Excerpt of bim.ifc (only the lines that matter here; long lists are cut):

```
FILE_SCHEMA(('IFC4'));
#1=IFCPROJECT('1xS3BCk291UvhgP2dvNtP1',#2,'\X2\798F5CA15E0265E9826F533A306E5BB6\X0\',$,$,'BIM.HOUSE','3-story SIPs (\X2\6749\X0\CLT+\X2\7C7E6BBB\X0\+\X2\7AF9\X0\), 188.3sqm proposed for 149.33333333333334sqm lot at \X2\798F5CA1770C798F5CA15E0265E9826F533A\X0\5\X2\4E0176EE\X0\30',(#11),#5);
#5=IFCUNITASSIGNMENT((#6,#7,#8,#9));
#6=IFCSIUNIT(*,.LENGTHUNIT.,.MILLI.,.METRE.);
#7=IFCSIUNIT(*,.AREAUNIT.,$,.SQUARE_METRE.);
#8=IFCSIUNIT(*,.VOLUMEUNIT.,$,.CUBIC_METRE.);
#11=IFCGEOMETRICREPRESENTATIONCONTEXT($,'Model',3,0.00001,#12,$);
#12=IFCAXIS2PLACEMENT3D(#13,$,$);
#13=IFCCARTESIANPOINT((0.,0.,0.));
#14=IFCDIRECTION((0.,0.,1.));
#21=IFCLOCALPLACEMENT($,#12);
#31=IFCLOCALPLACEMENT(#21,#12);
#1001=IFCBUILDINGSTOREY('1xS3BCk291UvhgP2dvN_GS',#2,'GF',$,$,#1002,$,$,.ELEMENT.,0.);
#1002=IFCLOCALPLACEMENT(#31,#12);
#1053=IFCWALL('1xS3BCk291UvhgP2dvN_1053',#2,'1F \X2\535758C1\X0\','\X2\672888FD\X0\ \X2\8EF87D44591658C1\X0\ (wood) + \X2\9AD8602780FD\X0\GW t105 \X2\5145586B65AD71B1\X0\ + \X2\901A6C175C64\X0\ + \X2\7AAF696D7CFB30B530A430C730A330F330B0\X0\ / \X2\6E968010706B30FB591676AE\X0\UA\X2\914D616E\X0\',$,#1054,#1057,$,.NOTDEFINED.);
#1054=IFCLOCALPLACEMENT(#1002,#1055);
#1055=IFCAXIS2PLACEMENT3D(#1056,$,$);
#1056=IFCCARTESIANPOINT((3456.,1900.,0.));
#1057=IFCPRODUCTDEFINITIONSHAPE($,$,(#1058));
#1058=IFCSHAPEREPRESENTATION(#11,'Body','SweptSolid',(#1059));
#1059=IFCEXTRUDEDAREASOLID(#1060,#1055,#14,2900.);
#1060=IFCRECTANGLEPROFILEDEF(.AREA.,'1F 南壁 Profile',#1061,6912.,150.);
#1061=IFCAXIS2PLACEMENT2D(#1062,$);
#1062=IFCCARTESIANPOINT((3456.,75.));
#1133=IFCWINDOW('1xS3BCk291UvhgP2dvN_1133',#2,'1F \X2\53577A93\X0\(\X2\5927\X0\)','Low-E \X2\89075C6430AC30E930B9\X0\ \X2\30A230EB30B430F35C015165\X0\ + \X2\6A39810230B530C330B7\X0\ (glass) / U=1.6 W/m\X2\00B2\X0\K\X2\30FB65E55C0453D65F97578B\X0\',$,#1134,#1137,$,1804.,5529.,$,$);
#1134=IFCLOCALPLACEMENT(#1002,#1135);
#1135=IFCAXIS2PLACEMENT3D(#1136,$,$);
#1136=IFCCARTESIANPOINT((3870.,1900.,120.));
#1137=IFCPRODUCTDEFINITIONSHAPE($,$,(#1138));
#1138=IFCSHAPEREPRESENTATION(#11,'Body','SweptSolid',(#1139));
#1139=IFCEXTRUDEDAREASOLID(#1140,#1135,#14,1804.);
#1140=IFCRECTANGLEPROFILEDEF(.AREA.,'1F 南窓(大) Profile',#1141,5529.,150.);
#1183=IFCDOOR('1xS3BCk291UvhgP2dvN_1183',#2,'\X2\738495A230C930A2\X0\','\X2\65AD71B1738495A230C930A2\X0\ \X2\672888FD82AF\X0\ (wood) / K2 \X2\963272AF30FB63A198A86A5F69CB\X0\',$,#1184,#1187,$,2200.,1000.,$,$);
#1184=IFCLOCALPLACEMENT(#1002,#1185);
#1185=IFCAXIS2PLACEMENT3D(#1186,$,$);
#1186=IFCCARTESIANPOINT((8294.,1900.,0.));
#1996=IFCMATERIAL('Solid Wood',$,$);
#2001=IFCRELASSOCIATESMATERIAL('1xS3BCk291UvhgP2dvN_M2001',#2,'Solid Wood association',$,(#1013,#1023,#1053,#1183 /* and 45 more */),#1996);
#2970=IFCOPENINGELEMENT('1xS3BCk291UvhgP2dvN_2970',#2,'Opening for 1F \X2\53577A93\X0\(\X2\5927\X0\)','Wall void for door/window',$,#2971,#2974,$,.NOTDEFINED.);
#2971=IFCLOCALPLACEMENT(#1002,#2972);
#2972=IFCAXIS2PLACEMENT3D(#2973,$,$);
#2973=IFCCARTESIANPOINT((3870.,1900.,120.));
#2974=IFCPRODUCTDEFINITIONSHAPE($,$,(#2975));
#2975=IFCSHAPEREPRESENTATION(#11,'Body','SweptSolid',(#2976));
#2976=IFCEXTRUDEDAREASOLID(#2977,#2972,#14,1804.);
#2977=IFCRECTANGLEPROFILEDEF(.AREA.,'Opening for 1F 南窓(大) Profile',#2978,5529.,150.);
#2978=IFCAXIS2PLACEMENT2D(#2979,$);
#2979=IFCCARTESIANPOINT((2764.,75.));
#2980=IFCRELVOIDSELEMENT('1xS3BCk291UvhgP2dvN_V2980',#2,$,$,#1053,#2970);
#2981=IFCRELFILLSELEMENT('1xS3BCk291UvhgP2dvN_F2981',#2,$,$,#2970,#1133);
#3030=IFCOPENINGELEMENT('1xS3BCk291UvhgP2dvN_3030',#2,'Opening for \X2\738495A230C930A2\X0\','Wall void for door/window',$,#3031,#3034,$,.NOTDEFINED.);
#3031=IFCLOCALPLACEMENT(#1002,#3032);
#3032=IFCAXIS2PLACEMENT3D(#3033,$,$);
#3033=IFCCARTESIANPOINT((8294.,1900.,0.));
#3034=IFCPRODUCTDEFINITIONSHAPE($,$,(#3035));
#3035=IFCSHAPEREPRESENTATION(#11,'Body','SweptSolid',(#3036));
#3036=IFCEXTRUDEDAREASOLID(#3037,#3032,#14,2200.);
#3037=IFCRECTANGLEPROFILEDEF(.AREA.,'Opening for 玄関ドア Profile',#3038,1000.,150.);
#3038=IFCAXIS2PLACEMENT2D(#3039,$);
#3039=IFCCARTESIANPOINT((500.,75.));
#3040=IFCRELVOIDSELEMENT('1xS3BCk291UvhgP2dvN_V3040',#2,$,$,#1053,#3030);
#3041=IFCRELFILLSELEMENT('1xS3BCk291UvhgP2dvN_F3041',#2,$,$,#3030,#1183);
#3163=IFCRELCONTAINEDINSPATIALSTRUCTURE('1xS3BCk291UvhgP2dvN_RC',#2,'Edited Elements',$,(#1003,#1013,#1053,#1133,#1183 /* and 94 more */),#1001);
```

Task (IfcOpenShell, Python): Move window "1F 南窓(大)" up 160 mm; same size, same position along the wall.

```python
import numpy as np
import ifcopenshell
import ifcopenshell.api.geometry
import ifcopenshell.util.placement
import ifcopenshell.util.unit

model = ifcopenshell.open("bim.ifc")
unit_scale = ifcopenshell.util.unit.calculate_unit_scale(model)

window = model.by_guid("1xS3BCk291UvhgP2dvN_1133")
opening = window.FillsVoids[0].RelatingOpeningElement
dz = 160.0

shift = np.array([0.0, 0.0, dz])
# The window is not placed relative to its opening, so move both.
for product in (opening, window):
    matrix = ifcopenshell.util.placement.get_local_placement(product.ObjectPlacement)
    matrix[:3, 3] += shift
    ifcopenshell.api.geometry.edit_object_placement(model, product=product, matrix=matrix, is_si=False)

print(f"moved by {dz * unit_scale:+.3f} m")

model.write("bim_edited.ifc")
```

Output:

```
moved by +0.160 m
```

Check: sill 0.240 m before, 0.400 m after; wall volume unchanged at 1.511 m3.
